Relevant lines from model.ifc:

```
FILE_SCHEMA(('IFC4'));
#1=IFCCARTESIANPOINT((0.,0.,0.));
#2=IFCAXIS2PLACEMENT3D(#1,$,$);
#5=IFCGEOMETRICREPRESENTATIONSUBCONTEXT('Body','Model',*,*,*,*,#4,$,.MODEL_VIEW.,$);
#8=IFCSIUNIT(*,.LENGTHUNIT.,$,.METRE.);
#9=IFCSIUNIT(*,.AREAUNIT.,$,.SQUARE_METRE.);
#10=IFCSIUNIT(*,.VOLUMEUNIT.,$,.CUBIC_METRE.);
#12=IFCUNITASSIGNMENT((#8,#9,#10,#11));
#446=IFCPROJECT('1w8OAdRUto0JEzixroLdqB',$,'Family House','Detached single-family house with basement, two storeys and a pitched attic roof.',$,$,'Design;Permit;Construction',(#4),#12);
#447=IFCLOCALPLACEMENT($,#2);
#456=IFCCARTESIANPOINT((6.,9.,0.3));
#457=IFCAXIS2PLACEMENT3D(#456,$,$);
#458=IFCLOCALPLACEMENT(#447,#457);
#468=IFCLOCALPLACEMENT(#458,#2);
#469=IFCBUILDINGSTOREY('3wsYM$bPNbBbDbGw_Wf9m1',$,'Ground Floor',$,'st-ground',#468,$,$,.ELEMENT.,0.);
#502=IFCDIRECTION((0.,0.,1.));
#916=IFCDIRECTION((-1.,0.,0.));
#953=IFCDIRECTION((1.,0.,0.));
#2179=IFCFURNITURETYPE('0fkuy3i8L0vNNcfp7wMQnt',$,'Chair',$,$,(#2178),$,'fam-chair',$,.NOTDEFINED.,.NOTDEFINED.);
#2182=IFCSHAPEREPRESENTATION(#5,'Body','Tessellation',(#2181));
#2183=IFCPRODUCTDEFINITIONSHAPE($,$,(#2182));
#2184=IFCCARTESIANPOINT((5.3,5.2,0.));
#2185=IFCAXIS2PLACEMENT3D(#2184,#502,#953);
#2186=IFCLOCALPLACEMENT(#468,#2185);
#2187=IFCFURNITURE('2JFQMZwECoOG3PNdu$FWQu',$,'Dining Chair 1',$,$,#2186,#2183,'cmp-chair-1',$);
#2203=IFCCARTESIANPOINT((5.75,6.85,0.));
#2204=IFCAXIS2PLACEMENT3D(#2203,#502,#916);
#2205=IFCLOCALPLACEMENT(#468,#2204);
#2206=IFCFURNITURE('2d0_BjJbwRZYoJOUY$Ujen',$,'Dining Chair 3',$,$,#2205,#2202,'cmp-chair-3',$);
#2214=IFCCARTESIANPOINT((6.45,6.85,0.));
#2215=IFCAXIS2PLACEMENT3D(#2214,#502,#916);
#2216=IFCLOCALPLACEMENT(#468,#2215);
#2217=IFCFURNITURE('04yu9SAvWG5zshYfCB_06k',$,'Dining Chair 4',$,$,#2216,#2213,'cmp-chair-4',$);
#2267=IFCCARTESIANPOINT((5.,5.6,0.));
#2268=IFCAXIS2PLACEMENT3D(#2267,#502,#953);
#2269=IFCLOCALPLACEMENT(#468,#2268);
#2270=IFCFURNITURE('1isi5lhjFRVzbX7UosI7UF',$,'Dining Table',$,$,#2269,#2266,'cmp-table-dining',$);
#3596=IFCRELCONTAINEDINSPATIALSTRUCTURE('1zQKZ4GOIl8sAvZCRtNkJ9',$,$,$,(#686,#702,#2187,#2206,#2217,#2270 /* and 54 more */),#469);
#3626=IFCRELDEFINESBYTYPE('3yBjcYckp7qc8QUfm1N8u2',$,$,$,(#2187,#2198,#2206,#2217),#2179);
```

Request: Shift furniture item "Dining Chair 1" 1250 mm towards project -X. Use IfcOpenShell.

```python
import ifcopenshell
import ifcopenshell.api.geometry
import ifcopenshell.util.placement
import ifcopenshell.util.unit

model = ifcopenshell.open("model.ifc")
unit_scale = ifcopenshell.util.unit.calculate_unit_scale(model)

item = model.by_id(2187)
matrix = ifcopenshell.util.placement.get_local_placement(item.ObjectPlacement)
matrix[0, 3] -= 1.25 / unit_scale
ifcopenshell.api.geometry.edit_object_placement(model, product=item, matrix=matrix, is_si=False)

print(ifcopenshell.util.placement.get_local_placement(item.ObjectPlacement).round(3) + 0.0)

model.write("model_rev.ifc")
```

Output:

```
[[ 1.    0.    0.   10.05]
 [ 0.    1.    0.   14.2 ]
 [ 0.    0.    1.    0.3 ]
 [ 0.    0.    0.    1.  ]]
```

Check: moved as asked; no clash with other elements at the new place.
